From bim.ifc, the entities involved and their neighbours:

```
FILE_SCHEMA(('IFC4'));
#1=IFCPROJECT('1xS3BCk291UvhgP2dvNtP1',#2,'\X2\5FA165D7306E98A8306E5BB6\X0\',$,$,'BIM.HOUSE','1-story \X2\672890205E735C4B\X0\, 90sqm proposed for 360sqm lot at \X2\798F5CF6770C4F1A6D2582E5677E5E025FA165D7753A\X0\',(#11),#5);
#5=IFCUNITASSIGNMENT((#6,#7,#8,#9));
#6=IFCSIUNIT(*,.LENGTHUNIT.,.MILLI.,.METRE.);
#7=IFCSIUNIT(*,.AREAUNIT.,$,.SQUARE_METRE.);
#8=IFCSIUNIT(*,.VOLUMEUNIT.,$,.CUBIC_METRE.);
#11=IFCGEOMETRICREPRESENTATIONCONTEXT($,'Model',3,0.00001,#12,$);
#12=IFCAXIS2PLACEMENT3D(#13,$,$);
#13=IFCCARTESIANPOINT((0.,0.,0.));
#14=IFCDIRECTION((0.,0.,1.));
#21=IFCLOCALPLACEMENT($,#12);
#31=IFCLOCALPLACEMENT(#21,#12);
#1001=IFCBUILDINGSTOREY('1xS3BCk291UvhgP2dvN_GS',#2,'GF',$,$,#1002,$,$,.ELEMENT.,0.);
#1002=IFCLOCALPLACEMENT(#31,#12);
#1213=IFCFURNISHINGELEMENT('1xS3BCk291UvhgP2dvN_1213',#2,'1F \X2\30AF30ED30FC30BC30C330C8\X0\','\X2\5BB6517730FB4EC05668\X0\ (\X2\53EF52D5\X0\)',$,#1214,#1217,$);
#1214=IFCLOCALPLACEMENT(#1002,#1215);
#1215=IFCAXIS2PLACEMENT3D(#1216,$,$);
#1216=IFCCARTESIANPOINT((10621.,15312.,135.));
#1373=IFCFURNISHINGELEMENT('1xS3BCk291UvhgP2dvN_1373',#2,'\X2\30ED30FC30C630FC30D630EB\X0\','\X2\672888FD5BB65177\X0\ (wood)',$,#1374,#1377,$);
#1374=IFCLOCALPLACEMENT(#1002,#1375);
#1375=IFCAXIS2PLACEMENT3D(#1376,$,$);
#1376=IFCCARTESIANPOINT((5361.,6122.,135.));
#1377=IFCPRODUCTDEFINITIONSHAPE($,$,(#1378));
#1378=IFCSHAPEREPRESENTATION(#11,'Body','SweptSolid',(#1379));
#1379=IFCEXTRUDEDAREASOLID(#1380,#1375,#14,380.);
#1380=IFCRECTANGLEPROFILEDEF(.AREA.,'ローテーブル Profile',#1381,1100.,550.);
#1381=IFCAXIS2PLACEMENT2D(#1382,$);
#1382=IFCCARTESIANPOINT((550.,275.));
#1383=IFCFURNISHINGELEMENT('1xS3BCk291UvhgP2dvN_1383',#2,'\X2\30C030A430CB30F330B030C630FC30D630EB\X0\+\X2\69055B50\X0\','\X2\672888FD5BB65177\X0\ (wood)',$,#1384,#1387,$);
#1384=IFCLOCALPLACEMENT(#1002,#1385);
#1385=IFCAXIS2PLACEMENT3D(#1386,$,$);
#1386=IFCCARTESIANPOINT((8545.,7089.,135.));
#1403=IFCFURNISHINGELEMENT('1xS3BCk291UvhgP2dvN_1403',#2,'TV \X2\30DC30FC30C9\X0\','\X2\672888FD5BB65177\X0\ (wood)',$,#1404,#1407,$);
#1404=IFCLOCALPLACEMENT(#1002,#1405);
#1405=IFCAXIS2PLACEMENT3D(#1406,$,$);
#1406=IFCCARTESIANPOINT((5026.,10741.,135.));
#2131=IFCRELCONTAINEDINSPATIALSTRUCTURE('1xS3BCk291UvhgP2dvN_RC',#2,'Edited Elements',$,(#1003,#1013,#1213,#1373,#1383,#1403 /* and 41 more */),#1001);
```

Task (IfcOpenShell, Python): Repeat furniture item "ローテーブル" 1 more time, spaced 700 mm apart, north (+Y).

```python
import numpy as np
import ifcopenshell
import ifcopenshell.api.geometry
import ifcopenshell.api.root
import ifcopenshell.util.element
import ifcopenshell.util.placement
import ifcopenshell.util.unit

model = ifcopenshell.open("bim.ifc")
unit_scale = ifcopenshell.util.unit.calculate_unit_scale(model)


def reuse_history(source, copy):
    """copy_class also copies each property set's owner history, people and application; keep the originals."""
    for rel in copy.IsDefinedBy:
        if rel.is_a("IfcRelDefinesByProperties") and (history := rel.RelatingPropertyDefinition.OwnerHistory):
            rel.RelatingPropertyDefinition.OwnerHistory = source.OwnerHistory
            ifcopenshell.util.element.remove_deep2(model, history)


source = model.by_guid("1xS3BCk291UvhgP2dvN_1373")
base = ifcopenshell.util.placement.get_local_placement(source.ObjectPlacement)
step = np.array([0.0, 1.0, 0.0]) * 0.7 / unit_scale

for i in range(1, 2):
    copy = ifcopenshell.api.root.copy_class(model, product=source)
    copy.Representation = ifcopenshell.util.element.copy_deep(
        model, source.Representation, exclude=["IfcGeometricRepresentationContext", "IfcRepresentationMap"]
    )
    reuse_history(source, copy)
    matrix = base.copy()
    matrix[:3, 3] += i * step
    print("added at", matrix[:3, 3].round(3) + 0.0)
    ifcopenshell.api.geometry.edit_object_placement(model, product=copy, matrix=matrix, is_si=False)

model.write("bim_v2.ifc")
```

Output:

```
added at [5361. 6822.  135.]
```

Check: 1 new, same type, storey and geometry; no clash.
